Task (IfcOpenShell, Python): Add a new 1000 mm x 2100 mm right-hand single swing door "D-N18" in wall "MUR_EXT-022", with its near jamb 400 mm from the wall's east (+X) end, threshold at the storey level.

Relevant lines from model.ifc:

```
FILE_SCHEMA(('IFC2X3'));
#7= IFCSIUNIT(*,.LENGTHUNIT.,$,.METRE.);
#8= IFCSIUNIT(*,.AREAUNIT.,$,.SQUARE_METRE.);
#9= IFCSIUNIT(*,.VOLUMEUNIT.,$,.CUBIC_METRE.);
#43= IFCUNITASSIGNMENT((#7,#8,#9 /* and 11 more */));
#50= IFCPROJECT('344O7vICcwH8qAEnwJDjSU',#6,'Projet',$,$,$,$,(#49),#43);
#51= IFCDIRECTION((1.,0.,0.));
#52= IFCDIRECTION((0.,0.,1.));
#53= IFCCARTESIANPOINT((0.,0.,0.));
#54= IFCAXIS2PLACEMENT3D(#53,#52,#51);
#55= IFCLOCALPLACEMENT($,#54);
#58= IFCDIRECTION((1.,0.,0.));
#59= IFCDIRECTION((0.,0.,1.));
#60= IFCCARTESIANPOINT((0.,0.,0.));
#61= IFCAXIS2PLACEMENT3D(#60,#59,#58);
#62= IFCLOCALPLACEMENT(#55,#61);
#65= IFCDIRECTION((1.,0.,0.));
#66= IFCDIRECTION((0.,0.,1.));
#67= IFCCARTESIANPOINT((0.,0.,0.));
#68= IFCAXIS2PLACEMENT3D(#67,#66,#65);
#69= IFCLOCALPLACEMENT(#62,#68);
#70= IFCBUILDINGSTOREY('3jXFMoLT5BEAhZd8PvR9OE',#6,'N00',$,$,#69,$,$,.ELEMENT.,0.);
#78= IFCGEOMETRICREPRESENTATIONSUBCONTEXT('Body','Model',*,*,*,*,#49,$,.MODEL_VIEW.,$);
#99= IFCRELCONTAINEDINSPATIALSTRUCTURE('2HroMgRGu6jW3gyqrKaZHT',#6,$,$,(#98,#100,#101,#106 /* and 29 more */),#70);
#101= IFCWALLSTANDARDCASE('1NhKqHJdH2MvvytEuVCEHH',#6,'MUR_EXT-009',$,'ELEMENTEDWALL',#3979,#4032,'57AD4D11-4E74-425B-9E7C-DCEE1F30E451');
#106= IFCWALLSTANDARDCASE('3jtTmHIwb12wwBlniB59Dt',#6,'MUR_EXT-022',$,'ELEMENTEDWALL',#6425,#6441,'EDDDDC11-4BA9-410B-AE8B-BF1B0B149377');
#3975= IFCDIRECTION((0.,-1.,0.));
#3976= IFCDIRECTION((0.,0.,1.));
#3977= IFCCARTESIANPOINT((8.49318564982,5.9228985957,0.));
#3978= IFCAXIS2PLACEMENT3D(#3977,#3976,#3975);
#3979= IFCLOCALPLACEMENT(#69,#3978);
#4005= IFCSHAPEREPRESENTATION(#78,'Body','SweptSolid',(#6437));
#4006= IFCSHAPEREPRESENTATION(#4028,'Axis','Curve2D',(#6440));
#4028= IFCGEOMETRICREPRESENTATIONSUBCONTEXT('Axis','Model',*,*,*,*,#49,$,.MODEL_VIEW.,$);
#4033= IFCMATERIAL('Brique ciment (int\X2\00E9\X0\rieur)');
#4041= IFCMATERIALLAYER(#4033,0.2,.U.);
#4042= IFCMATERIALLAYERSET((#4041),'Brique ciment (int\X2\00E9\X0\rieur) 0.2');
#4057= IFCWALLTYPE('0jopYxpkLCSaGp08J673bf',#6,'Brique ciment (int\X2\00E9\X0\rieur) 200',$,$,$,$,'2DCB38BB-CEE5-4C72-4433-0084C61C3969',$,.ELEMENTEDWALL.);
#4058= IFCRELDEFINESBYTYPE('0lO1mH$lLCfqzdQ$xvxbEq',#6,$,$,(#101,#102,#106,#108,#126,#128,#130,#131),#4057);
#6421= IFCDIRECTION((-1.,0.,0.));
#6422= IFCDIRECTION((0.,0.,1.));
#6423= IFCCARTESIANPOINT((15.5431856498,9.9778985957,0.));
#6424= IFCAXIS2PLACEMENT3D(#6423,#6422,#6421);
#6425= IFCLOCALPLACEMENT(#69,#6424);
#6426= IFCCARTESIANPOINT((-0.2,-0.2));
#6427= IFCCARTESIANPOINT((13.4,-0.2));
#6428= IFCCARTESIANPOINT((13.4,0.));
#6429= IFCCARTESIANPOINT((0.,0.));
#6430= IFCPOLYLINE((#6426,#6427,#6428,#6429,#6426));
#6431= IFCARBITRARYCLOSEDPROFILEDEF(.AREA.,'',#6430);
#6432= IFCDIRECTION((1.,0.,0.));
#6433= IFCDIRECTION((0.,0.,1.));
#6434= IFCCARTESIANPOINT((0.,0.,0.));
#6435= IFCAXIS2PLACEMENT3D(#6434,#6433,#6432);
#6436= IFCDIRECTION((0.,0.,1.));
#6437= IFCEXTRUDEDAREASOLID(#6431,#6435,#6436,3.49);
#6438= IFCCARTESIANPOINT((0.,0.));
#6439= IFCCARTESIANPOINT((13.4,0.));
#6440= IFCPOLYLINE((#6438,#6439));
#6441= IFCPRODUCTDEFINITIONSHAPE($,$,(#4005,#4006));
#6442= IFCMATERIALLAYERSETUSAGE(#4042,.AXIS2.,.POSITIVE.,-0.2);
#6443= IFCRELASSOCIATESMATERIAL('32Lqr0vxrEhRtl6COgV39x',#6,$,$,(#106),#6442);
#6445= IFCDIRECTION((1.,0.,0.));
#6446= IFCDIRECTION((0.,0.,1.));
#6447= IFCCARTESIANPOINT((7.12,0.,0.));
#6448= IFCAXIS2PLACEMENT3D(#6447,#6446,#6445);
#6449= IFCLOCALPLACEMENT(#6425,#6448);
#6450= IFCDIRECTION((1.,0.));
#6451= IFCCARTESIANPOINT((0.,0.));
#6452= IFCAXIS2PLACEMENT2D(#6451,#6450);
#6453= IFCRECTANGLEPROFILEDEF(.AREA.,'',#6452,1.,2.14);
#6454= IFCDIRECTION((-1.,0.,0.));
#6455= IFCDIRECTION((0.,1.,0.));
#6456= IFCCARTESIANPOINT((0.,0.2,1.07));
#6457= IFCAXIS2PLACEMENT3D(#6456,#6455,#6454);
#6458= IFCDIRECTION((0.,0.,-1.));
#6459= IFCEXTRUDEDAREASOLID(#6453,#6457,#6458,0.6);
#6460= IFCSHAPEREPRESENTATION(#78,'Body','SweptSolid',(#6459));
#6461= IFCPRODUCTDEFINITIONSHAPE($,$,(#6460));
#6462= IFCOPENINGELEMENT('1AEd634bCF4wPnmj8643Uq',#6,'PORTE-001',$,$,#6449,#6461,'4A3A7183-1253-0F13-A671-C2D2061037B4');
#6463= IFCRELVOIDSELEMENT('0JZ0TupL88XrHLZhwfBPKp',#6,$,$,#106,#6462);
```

```python
import numpy as np
import ifcopenshell
import ifcopenshell.api.feature
import ifcopenshell.api.geometry
import ifcopenshell.api.root
import ifcopenshell.api.spatial
import ifcopenshell.api.type
import ifcopenshell.geom
import ifcopenshell.util.element
import ifcopenshell.util.placement
import ifcopenshell.util.representation
import ifcopenshell.util.shape
import ifcopenshell.util.unit

model = ifcopenshell.open("model.ifc")
unit_scale = ifcopenshell.util.unit.calculate_unit_scale(model)
settings = ifcopenshell.geom.settings()


def volume(element):
    """Net volume in cubic metres, openings subtracted."""
    shape = ifcopenshell.geom.create_shape(settings, element)
    return ifcopenshell.util.shape.get_volume(shape.geometry)


wall = model.by_guid("3jtTmHIwb12wwBlniB59Dt")
storey = ifcopenshell.util.element.get_container(wall, ifc_class="IfcBuildingStorey")
context = ifcopenshell.util.representation.get_context(model, "Model", "Body", "MODEL_VIEW")
before = volume(wall)

width, height, from_end, sill = 1, 2.1, 0.4, 0.0  # metres

# The wall runs along its own X axis, and the end named is its -X end.
wall_shape = ifcopenshell.geom.create_shape(settings, wall)
x, y, z = ifcopenshell.util.shape.get_vertices(wall_shape.geometry).T
start = x.min() + from_end
face, thickness = float(y.min()), float(y.max() - y.min())
wall_matrix = ifcopenshell.util.placement.get_local_placement(wall.ObjectPlacement)
level = ifcopenshell.util.placement.get_local_placement(storey.ObjectPlacement)[2, 3]


def in_wall(x, y):
    """Placement at x, y metres in the wall's axes, at sill height."""
    matrix = wall_matrix.copy()
    matrix[:, 3] = wall_matrix @ np.array([x / unit_scale, y / unit_scale, 0.0, 1.0])
    matrix[2, 3] = level + sill / unit_scale
    return matrix


# Opening: a box that overshoots both wall faces by 50 mm.
opening = ifcopenshell.api.root.create_entity(model, ifc_class="IfcOpeningElement")
box = ifcopenshell.api.geometry.add_wall_representation(
    model, context=context, length=width, height=height, thickness=thickness + 0.1
)
ifcopenshell.api.geometry.assign_representation(model, product=opening, representation=box)
ifcopenshell.api.geometry.edit_object_placement(model, product=opening, matrix=in_wall(start, face - 0.05), is_si=False)
ifcopenshell.api.feature.add_feature(model, feature=opening, element=wall)

door = ifcopenshell.api.root.create_entity(model, ifc_class="IfcDoor", name="D-N18")
door.OverallWidth, door.OverallHeight = width / unit_scale, height / unit_scale
body = ifcopenshell.api.geometry.add_door_representation(
    model,
    context=context,
    overall_width=door.OverallWidth,
    overall_height=door.OverallHeight,
    operation_type="SINGLE_SWING_RIGHT",
    lining_properties={"LiningDepth": thickness / unit_scale, "ThresholdDepth": thickness / unit_scale},
)
ifcopenshell.api.geometry.assign_representation(model, product=door, representation=body)
ifcopenshell.api.spatial.assign_container(model, products=[door], relating_structure=storey)
fills = ifcopenshell.api.feature.add_filling(model, opening=opening, element=door)
fills.OwnerHistory = door.OwnerHistory  # required in IFC2X3

# IFC2X3 keeps the operation on the door style.
style = ifcopenshell.api.root.create_entity(model, ifc_class="IfcDoorStyle", name="D-N18")
style.OperationType, style.ConstructionType = "SINGLE_SWING_RIGHT", "NOTDEFINED"
style.ParameterTakesPrecedence = style.Sizeable = False
ifcopenshell.api.type.assign_type(model, related_objects=[door], relating_type=style)

# The lining spans the wall, so the door starts at the wall face.
ifcopenshell.api.geometry.edit_object_placement(model, product=door, matrix=in_wall(start, face), is_si=False)

after = volume(wall)

print(f"wall volume {before:.3f} -> {after:.3f} m3")

model.write("model_updated.ifc")
```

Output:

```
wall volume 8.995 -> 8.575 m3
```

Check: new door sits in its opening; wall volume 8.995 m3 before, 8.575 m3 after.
